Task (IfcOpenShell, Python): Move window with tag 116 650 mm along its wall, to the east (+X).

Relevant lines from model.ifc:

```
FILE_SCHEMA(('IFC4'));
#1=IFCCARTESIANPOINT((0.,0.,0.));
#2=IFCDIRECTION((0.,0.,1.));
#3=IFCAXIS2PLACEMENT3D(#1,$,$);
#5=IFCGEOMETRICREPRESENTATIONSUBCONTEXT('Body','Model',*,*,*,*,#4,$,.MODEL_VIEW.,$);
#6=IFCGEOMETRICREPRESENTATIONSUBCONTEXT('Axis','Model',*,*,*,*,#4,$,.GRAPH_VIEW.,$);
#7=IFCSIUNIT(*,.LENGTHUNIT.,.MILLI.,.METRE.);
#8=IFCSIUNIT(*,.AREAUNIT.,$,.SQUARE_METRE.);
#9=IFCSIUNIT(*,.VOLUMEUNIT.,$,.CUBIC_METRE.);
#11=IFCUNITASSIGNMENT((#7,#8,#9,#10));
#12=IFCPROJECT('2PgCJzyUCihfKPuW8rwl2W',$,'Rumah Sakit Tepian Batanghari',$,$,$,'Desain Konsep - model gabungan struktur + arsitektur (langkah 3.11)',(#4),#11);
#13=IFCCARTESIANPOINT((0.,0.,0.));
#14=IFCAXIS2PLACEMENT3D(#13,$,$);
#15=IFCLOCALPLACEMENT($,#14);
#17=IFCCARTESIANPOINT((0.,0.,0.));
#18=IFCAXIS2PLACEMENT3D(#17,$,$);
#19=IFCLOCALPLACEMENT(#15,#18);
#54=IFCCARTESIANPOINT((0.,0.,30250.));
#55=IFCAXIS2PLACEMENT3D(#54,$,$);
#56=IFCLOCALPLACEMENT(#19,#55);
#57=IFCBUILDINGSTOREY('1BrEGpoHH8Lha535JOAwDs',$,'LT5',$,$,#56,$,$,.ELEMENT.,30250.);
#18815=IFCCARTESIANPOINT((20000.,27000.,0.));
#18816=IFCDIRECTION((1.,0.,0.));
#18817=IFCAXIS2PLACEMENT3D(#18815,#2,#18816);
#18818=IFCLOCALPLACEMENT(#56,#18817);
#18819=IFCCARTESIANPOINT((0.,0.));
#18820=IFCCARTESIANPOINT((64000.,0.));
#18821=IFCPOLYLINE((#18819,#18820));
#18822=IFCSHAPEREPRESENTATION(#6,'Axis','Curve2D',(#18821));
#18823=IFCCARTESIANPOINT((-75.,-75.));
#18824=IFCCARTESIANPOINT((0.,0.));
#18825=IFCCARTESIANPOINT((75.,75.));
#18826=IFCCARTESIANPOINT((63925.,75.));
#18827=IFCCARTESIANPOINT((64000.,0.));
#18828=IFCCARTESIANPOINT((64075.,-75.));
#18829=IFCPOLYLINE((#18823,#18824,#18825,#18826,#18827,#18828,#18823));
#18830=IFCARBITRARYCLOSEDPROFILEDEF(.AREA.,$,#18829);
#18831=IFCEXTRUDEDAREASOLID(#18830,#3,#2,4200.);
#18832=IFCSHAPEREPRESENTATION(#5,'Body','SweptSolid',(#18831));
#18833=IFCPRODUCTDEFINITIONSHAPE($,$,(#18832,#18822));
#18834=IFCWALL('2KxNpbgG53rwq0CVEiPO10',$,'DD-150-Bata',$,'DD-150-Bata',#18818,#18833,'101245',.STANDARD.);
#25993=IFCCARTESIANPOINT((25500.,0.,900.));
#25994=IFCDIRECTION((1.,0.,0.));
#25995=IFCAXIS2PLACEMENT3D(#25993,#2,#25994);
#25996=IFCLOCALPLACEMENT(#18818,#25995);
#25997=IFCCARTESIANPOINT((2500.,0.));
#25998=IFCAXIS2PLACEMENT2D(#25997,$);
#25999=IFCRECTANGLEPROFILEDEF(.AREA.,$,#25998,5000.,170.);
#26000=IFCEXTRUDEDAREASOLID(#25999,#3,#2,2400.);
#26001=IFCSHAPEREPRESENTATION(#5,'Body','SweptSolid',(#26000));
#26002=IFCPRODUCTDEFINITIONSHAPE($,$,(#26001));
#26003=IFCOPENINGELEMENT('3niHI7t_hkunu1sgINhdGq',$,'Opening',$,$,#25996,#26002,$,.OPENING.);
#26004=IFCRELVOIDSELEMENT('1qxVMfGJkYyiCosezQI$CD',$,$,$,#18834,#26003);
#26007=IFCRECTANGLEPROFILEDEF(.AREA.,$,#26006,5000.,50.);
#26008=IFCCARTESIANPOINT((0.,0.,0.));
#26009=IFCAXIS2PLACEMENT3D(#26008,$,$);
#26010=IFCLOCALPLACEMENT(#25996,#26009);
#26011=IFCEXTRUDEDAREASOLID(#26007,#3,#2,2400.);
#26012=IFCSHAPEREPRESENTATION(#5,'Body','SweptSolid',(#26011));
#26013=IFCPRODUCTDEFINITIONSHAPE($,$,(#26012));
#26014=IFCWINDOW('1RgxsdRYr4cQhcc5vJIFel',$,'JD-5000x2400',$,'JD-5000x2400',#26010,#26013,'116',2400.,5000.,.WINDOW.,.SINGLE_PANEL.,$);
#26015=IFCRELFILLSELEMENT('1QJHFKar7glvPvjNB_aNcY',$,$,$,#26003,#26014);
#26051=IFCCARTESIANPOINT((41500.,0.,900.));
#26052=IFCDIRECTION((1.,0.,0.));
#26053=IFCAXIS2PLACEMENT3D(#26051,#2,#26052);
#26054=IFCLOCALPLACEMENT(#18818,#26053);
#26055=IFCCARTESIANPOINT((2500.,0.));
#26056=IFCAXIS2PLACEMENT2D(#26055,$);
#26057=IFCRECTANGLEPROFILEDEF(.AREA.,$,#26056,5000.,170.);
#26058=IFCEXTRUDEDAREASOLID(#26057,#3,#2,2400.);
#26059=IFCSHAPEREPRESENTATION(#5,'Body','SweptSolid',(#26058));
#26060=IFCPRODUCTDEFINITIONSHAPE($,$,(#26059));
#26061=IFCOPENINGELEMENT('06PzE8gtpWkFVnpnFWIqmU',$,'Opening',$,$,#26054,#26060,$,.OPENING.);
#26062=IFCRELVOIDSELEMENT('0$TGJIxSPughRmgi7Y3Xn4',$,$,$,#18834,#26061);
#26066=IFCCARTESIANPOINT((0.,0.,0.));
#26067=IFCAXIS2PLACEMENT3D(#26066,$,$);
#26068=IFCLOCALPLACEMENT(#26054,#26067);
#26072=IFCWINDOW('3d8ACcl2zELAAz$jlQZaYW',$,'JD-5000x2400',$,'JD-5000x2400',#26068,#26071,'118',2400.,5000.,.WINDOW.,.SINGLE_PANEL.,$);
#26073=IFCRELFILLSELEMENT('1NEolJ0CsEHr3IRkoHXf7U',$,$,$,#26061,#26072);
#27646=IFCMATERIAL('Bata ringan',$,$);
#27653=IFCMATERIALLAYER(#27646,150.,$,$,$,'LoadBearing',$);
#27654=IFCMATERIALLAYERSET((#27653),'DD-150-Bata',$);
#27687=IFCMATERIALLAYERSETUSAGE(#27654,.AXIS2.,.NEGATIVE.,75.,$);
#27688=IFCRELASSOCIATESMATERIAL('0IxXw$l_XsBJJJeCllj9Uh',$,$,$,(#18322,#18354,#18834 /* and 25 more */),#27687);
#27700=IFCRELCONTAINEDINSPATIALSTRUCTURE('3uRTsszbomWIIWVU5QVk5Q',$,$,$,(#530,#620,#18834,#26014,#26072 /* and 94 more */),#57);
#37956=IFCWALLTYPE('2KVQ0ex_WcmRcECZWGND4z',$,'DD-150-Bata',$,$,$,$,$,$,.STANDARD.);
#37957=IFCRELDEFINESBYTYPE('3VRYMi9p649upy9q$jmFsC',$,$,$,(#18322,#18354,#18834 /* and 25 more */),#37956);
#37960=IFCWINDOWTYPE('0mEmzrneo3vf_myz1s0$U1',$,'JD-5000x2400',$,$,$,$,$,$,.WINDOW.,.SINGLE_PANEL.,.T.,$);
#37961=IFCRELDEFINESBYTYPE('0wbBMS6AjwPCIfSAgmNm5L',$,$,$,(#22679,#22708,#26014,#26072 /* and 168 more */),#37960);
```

```python
import ifcopenshell
import ifcopenshell.api.geometry
import ifcopenshell.util.placement

model = ifcopenshell.open("model.ifc")

window = model.by_guid("1RgxsdRYr4cQhcc5vJIFel")
opening = window.FillsVoids[0].RelatingOpeningElement
wall = opening.VoidsElements[0].RelatingBuildingElement

wall_matrix = ifcopenshell.util.placement.get_local_placement(wall.ObjectPlacement)
shift = wall_matrix[:3, 0] * 650.0
before = ifcopenshell.util.placement.get_local_placement(window.ObjectPlacement)[:3, 3].copy()

# The window is placed relative to its opening, so it follows when the opening moves.
matrix = ifcopenshell.util.placement.get_local_placement(opening.ObjectPlacement)
matrix[:3, 3] += shift
ifcopenshell.api.geometry.edit_object_placement(
    model, product=opening, matrix=matrix, is_si=False, should_transform_children=True
)

after = ifcopenshell.util.placement.get_local_placement(window.ObjectPlacement)[:3, 3]
print("window moved by", (after - before).round(3) + 0.0)

model.write("model_updated.ifc")
```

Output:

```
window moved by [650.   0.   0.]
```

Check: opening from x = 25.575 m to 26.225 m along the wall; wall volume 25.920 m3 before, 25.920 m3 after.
